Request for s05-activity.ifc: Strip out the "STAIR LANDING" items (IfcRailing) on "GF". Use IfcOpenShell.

First a look at what the model holds.

```python
import ifcopenshell
import ifcopenshell.util.element

model = ifcopenshell.open("s05-activity.ifc")
print(model.schema)
storey = next(s for s in model.by_type("IfcBuildingStorey") if s.Name == "GF")
railings = [e for e in ifcopenshell.util.element.get_decomposition(storey) if e.is_a("IfcRailing")]
seen = {}
for e in railings:
    element_type = ifcopenshell.util.element.get_type(e)
    name = element_type.Name if element_type not in (None, e) else None
    seen[name] = seen.get(name, 0) + 1
for name, count in sorted(seen.items(), key=str):
    print(count, "x", name)
```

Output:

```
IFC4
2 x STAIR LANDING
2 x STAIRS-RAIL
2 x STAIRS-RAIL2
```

```python
import ifcopenshell
import ifcopenshell.api.root
import ifcopenshell.util.element

model = ifcopenshell.open("s05-activity.ifc")

storey = next(s for s in model.by_type("IfcBuildingStorey") if s.Name == "GF")
railings = [e for e in ifcopenshell.util.element.get_decomposition(storey) if e.is_a("IfcRailing")]
targets = [e for e in railings if (t := ifcopenshell.util.element.get_type(e)) not in (None, e) and t.Name == "STAIR LANDING"]

for e in targets:
    ifcopenshell.api.root.remove_product(model, product=e)
print(len(targets), "removed")

model.write("s05-activity_updated.ifc")
```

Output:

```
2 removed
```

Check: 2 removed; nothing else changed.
